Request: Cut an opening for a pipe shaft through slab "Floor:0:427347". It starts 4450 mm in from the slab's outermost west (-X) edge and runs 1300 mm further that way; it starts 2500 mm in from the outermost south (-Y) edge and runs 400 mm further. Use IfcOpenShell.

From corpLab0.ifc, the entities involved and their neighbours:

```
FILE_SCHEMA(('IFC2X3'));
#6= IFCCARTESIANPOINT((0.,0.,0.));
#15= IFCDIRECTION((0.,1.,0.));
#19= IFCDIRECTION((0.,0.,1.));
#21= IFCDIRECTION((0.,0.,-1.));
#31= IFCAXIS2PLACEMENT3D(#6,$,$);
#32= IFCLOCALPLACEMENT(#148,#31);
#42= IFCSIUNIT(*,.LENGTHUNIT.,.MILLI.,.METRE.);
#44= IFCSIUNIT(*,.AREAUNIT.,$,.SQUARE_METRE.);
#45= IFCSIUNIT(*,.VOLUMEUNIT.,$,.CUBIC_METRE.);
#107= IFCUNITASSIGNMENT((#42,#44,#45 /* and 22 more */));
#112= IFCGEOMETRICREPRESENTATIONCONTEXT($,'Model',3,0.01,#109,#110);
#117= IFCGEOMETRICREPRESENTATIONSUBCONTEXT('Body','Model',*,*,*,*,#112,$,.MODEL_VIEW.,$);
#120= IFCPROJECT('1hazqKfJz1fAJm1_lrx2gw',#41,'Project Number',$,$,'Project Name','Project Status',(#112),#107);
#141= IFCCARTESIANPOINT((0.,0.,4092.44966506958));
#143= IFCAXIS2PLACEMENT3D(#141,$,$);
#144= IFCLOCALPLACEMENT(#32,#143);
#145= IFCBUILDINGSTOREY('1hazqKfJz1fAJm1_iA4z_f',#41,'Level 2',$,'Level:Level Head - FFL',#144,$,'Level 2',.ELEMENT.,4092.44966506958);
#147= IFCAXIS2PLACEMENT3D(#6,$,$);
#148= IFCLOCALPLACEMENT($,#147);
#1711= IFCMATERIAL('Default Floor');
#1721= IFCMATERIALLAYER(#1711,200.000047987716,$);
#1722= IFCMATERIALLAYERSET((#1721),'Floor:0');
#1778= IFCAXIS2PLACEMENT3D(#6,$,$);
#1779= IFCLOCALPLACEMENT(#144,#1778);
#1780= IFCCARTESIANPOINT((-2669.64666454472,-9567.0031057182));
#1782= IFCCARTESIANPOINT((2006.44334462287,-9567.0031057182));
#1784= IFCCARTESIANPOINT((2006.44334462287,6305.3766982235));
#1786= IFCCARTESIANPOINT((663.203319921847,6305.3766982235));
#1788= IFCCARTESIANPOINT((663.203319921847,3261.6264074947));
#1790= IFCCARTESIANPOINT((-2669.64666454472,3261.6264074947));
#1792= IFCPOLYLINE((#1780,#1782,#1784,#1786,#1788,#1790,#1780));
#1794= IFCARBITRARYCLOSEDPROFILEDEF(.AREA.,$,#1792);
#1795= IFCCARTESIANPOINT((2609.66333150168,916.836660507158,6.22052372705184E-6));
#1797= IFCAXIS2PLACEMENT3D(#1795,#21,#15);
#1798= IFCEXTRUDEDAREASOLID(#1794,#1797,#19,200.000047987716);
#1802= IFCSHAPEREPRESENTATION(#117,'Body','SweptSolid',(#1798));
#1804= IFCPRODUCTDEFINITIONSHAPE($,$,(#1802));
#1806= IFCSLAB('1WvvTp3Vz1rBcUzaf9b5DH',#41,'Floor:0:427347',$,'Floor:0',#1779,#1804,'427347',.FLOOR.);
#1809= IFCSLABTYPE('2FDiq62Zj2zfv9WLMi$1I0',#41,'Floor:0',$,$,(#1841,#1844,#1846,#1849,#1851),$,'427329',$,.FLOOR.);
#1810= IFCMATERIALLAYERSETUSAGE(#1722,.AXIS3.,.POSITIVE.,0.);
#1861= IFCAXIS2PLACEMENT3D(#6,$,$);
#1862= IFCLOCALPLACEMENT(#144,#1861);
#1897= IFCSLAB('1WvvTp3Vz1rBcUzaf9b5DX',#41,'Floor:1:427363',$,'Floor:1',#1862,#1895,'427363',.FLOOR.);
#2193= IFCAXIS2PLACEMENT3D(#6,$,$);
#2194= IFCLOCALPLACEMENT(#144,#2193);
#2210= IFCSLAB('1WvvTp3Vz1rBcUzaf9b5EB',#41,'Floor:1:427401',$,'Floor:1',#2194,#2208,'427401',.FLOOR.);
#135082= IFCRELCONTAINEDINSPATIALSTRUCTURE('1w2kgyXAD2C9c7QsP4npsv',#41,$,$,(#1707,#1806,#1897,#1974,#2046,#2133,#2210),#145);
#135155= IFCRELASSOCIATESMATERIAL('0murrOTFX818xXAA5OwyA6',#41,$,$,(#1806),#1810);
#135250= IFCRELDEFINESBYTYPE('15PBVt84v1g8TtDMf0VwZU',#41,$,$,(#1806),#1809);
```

```python
import numpy as np
import ifcopenshell
import ifcopenshell.api.feature
import ifcopenshell.api.geometry
import ifcopenshell.api.root
import ifcopenshell.geom
import ifcopenshell.util.placement
import ifcopenshell.util.representation
import ifcopenshell.util.shape
import ifcopenshell.util.unit

model = ifcopenshell.open("corpLab0.ifc")
unit_scale = ifcopenshell.util.unit.calculate_unit_scale(model)
settings = ifcopenshell.geom.settings()


def volume(element):
    """Net volume in cubic metres, openings subtracted."""
    shape = ifcopenshell.geom.create_shape(settings, element)
    return ifcopenshell.util.shape.get_volume(shape.geometry)


slab = model.by_guid("1WvvTp3Vz1rBcUzaf9b5DH")
before = volume(slab)

# Extent in the slab's own axes, in metres. The edges named are its -X and -Y sides.
slab_shape = ifcopenshell.geom.create_shape(settings, slab)
vertices = ifcopenshell.util.shape.get_vertices(slab_shape.geometry)
x_min, y_min, bottom = vertices.min(axis=0)
top = vertices[:, 2].max()

opening = ifcopenshell.api.root.create_entity(model, ifc_class="IfcOpeningElement", name="Pipe shaft opening")
context = ifcopenshell.util.representation.get_context(model, "Model", "Body", "MODEL_VIEW")
width, depth = 1.3, 0.4
outline = [(0.0, 0.0), (width, 0.0), (width, depth), (0.0, depth), (0.0, 0.0)]
# Overshoot both faces by 50 mm so the cut is clean.
shape = ifcopenshell.api.geometry.add_slab_representation(
    model, context=context, depth=top - bottom + 0.1, polyline=outline
)
ifcopenshell.api.geometry.assign_representation(model, product=opening, representation=shape)

matrix = ifcopenshell.util.placement.get_local_placement(slab.ObjectPlacement)
matrix[:, 3] = matrix @ np.append(np.array([x_min + 4.45, y_min + 2.5, bottom - 0.05]) / unit_scale, 1.0)
ifcopenshell.api.geometry.edit_object_placement(model, product=opening, matrix=matrix, is_si=False)
ifcopenshell.api.feature.add_feature(model, feature=opening, element=slab)

after = volume(slab)

print(f"slab volume {before:.3f} -> {after:.3f} m3")

model.write("corpLab0_edited.ifc")
```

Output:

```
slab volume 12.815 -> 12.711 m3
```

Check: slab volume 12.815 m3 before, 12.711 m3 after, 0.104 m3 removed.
